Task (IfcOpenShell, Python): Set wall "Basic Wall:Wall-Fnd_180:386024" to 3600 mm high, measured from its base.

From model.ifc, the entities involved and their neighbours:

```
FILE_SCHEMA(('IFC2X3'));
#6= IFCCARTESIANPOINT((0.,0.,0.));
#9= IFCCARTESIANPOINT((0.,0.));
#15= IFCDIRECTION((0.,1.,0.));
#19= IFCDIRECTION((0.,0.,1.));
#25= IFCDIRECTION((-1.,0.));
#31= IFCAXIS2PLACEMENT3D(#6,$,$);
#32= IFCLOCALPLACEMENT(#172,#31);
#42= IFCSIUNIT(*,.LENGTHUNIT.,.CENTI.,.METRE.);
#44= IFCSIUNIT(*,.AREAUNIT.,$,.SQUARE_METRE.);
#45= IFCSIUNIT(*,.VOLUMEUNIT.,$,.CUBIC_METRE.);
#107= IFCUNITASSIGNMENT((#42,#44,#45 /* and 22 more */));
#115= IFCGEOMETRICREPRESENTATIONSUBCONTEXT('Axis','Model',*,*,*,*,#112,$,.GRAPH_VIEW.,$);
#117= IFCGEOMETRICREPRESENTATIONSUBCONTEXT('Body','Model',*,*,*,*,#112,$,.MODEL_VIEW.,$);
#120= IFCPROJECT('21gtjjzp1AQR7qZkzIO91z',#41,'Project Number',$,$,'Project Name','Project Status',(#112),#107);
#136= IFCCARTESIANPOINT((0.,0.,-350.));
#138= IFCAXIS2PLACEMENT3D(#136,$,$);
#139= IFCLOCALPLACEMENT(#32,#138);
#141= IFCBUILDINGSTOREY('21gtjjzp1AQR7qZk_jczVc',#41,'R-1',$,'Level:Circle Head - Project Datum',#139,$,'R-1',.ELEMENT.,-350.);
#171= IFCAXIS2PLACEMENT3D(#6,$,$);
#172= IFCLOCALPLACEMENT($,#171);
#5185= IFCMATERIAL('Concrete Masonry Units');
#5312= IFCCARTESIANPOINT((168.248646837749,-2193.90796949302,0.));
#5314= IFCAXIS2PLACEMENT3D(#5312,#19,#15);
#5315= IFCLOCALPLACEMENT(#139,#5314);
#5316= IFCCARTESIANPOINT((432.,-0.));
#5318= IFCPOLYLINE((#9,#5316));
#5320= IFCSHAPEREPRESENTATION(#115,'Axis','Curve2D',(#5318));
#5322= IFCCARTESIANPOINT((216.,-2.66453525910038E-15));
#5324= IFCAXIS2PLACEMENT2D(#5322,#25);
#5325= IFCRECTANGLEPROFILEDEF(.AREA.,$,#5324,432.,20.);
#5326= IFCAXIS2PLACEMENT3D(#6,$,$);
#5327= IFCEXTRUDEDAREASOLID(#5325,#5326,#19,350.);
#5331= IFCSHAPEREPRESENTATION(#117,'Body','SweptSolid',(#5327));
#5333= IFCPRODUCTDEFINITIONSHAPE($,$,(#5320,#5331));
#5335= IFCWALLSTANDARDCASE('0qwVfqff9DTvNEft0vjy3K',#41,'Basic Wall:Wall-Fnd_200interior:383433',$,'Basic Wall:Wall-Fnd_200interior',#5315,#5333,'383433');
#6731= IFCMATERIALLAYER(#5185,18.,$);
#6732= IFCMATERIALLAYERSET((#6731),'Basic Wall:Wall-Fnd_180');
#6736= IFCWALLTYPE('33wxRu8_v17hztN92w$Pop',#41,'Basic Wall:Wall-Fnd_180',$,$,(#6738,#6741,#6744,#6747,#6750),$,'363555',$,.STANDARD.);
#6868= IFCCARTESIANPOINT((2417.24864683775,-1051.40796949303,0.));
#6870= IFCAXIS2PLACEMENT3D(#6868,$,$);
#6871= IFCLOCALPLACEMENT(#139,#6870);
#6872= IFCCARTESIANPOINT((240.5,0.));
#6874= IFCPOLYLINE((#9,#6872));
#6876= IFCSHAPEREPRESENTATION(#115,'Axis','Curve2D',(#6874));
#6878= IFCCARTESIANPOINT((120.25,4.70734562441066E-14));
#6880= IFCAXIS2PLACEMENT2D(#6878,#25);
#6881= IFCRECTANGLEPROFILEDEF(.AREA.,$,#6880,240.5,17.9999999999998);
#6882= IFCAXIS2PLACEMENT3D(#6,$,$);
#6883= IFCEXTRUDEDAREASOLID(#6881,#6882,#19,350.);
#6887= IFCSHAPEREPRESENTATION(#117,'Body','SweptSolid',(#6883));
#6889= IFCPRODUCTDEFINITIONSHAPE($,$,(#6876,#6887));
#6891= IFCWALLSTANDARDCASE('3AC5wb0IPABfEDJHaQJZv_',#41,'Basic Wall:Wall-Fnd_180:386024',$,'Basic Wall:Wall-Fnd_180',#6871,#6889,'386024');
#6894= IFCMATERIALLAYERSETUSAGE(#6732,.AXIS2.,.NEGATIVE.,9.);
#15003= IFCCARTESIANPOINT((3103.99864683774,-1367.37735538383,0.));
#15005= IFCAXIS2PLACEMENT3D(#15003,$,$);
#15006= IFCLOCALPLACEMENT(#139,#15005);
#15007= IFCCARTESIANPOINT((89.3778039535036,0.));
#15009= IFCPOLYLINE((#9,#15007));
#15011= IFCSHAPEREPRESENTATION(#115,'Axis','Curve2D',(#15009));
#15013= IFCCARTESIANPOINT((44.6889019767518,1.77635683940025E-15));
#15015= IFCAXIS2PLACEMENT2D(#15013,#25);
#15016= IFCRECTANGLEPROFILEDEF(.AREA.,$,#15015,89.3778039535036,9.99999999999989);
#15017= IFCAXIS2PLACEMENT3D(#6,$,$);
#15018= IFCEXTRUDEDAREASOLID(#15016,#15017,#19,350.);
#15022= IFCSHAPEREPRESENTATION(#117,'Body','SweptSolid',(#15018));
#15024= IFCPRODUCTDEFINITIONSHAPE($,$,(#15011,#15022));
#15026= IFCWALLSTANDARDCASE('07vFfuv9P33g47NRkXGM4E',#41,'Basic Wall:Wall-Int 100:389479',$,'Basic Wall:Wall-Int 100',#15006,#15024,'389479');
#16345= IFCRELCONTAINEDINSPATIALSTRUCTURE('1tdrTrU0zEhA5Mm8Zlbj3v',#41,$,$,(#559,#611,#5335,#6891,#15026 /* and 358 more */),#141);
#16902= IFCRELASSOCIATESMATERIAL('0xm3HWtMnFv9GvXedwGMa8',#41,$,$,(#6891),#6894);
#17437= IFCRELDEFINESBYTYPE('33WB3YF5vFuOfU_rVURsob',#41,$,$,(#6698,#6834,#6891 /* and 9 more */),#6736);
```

```python
import ifcopenshell
import ifcopenshell.geom
import ifcopenshell.util.representation
import ifcopenshell.util.shape
import ifcopenshell.util.unit

model = ifcopenshell.open("model.ifc")
unit_scale = ifcopenshell.util.unit.calculate_unit_scale(model)
settings = ifcopenshell.geom.settings()


def volume(element):
    """Net volume in cubic metres, openings subtracted."""
    shape = ifcopenshell.geom.create_shape(settings, element)
    return ifcopenshell.util.shape.get_volume(shape.geometry)


wall = model.by_guid("3AC5wb0IPABfEDJHaQJZv_")
before = volume(wall)

body = ifcopenshell.util.representation.get_representation(wall, "Model", "Body")
solid = body.Items[0]
old_height = solid.Depth
solid.Depth = 3.6 / unit_scale
after = volume(wall)

print(f"height {old_height:g} -> {solid.Depth:g}, volume {before:.3f} -> {after:.3f} m3")

model.write("model_updated.ifc")
```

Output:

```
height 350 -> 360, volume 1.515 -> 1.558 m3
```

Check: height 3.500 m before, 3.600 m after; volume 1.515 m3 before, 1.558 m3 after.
